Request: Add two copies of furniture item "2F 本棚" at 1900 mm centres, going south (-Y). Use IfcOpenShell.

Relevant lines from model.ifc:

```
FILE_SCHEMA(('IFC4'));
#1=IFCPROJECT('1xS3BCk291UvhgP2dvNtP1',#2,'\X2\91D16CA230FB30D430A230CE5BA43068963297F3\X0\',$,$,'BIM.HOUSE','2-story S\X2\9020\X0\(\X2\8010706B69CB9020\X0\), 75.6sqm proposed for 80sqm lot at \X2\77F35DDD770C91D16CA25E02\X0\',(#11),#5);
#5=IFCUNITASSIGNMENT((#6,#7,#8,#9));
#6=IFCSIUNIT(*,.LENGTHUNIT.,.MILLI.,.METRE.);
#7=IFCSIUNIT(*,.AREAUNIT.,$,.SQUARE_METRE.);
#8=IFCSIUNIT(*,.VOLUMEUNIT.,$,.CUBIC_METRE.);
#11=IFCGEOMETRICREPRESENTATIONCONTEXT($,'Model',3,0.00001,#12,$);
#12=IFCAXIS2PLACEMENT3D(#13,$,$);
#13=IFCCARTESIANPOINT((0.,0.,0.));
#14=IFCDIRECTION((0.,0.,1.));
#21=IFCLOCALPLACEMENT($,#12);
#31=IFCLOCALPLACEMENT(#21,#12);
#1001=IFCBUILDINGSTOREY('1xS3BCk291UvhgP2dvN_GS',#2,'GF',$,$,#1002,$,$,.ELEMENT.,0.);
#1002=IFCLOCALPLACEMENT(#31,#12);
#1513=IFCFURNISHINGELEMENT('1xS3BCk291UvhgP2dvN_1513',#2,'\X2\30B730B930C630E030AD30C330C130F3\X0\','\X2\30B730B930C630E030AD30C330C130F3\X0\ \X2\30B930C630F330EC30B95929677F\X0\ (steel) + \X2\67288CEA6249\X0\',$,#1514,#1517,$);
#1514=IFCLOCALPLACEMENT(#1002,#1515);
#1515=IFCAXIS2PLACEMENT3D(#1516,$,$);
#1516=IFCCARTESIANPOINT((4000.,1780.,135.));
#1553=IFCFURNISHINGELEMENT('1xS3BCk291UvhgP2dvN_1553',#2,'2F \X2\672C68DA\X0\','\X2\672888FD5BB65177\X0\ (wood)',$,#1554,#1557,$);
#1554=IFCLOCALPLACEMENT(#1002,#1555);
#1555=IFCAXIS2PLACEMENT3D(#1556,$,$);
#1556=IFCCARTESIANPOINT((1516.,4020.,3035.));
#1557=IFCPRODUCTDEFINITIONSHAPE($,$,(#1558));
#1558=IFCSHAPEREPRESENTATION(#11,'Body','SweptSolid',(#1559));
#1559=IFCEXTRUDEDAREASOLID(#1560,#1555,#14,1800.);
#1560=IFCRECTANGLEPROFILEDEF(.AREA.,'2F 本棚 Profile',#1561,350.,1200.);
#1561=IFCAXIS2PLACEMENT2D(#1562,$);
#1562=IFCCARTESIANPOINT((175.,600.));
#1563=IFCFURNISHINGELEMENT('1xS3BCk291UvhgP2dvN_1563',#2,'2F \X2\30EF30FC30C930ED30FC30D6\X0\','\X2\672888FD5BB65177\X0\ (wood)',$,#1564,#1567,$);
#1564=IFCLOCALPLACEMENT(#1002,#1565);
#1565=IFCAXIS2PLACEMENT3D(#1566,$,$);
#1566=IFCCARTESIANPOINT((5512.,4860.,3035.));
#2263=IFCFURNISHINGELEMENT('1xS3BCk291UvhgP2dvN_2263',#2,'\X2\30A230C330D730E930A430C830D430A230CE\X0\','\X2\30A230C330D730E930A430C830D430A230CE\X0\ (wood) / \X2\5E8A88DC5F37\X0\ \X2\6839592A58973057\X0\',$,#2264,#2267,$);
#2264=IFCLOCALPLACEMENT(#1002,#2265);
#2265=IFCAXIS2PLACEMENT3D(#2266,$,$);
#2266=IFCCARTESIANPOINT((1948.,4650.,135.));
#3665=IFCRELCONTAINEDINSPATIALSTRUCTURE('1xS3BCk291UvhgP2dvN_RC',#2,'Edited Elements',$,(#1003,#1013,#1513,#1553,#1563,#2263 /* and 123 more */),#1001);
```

```python
import numpy as np
import ifcopenshell
import ifcopenshell.api.geometry
import ifcopenshell.api.root
import ifcopenshell.util.element
import ifcopenshell.util.placement

model = ifcopenshell.open("model.ifc")


def reuse_history(source, copy):
    """copy_class also copies each property set's owner history, people and application; keep the originals."""
    for rel in copy.IsDefinedBy:
        if rel.is_a("IfcRelDefinesByProperties") and (history := rel.RelatingPropertyDefinition.OwnerHistory):
            rel.RelatingPropertyDefinition.OwnerHistory = source.OwnerHistory
            ifcopenshell.util.element.remove_deep2(model, history)


source = model.by_id(1553)
base = ifcopenshell.util.placement.get_local_placement(source.ObjectPlacement)
step = np.array([0.0, -1.0, 0.0]) * 1900.0

for i in range(1, 3):
    copy = ifcopenshell.api.root.copy_class(model, product=source)
    copy.Representation = ifcopenshell.util.element.copy_deep(
        model, source.Representation, exclude=["IfcGeometricRepresentationContext", "IfcRepresentationMap"]
    )
    reuse_history(source, copy)
    matrix = base.copy()
    matrix[:3, 3] += i * step
    print("added at", matrix[:3, 3].round(3) + 0.0)
    ifcopenshell.api.geometry.edit_object_placement(model, product=copy, matrix=matrix, is_si=False)

model.write("model_updated.ifc")
```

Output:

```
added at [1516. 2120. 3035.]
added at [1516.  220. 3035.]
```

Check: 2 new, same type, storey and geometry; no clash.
